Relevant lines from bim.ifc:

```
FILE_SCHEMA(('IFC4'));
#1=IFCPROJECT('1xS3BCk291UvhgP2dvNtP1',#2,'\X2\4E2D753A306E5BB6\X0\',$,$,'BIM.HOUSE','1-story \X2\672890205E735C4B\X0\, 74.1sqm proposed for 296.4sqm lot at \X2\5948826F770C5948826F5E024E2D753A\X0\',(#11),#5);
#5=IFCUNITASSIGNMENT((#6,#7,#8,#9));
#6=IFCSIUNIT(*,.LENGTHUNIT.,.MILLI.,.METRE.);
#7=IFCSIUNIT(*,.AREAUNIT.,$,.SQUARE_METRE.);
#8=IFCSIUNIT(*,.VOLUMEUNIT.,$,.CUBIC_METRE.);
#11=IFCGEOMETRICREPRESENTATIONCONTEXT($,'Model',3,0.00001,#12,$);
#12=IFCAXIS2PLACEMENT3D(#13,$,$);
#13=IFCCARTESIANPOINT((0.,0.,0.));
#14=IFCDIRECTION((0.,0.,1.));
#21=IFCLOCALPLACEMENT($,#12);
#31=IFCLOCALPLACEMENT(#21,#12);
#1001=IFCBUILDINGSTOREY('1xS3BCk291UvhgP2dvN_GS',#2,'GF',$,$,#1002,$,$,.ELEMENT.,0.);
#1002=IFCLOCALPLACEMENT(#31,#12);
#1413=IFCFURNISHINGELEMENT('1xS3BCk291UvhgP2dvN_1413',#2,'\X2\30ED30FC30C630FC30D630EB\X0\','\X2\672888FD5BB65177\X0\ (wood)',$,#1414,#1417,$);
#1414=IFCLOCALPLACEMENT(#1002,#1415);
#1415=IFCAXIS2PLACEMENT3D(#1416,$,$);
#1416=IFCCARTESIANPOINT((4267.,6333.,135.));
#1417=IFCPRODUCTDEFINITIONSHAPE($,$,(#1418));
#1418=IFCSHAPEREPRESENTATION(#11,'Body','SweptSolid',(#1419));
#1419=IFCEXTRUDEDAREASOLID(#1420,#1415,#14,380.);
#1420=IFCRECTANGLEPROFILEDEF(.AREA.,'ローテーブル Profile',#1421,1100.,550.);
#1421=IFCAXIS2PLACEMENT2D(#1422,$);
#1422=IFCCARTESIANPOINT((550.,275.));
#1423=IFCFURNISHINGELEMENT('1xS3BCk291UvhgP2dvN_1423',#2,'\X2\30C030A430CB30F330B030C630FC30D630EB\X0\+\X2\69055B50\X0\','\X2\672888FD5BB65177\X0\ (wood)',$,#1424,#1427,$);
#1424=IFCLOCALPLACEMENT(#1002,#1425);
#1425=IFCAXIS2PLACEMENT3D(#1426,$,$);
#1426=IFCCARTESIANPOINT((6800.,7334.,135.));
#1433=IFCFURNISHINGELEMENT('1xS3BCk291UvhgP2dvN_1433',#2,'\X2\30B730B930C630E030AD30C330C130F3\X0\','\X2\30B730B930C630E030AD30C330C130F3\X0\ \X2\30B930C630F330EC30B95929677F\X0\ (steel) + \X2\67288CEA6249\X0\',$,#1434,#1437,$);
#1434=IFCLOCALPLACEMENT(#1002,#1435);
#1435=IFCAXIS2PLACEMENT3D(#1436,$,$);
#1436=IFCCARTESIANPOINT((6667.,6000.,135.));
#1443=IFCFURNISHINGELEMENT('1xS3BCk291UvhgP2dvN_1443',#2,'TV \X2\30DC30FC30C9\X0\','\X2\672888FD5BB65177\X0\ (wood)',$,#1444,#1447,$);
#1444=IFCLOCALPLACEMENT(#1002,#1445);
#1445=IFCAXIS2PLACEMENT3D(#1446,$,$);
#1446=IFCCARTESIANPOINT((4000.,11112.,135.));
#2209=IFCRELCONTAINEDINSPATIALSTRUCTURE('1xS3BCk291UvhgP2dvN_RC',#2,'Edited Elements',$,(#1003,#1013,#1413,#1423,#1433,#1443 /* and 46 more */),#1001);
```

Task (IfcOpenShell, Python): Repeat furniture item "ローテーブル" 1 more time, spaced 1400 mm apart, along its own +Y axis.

```python
import ifcopenshell
import ifcopenshell.api.geometry
import ifcopenshell.api.root
import ifcopenshell.util.element
import ifcopenshell.util.placement
import ifcopenshell.util.unit

model = ifcopenshell.open("bim.ifc")
unit_scale = ifcopenshell.util.unit.calculate_unit_scale(model)


def reuse_history(source, copy):
    """copy_class also copies each property set's owner history, people and application; keep the originals."""
    for rel in copy.IsDefinedBy:
        if rel.is_a("IfcRelDefinesByProperties") and (history := rel.RelatingPropertyDefinition.OwnerHistory):
            rel.RelatingPropertyDefinition.OwnerHistory = source.OwnerHistory
            ifcopenshell.util.element.remove_deep2(model, history)


source = model.by_guid("1xS3BCk291UvhgP2dvN_1413")
base = ifcopenshell.util.placement.get_local_placement(source.ObjectPlacement)
step = base[:3, 1] * 1.4 / unit_scale

for i in range(1, 2):
    copy = ifcopenshell.api.root.copy_class(model, product=source)
    copy.Representation = ifcopenshell.util.element.copy_deep(
        model, source.Representation, exclude=["IfcGeometricRepresentationContext", "IfcRepresentationMap"]
    )
    reuse_history(source, copy)
    matrix = base.copy()
    matrix[:3, 3] += i * step
    print("added at", matrix[:3, 3].round(3) + 0.0)
    ifcopenshell.api.geometry.edit_object_placement(model, product=copy, matrix=matrix, is_si=False)

model.write("bim_edited.ifc")
```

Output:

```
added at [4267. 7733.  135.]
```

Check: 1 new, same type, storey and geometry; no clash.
